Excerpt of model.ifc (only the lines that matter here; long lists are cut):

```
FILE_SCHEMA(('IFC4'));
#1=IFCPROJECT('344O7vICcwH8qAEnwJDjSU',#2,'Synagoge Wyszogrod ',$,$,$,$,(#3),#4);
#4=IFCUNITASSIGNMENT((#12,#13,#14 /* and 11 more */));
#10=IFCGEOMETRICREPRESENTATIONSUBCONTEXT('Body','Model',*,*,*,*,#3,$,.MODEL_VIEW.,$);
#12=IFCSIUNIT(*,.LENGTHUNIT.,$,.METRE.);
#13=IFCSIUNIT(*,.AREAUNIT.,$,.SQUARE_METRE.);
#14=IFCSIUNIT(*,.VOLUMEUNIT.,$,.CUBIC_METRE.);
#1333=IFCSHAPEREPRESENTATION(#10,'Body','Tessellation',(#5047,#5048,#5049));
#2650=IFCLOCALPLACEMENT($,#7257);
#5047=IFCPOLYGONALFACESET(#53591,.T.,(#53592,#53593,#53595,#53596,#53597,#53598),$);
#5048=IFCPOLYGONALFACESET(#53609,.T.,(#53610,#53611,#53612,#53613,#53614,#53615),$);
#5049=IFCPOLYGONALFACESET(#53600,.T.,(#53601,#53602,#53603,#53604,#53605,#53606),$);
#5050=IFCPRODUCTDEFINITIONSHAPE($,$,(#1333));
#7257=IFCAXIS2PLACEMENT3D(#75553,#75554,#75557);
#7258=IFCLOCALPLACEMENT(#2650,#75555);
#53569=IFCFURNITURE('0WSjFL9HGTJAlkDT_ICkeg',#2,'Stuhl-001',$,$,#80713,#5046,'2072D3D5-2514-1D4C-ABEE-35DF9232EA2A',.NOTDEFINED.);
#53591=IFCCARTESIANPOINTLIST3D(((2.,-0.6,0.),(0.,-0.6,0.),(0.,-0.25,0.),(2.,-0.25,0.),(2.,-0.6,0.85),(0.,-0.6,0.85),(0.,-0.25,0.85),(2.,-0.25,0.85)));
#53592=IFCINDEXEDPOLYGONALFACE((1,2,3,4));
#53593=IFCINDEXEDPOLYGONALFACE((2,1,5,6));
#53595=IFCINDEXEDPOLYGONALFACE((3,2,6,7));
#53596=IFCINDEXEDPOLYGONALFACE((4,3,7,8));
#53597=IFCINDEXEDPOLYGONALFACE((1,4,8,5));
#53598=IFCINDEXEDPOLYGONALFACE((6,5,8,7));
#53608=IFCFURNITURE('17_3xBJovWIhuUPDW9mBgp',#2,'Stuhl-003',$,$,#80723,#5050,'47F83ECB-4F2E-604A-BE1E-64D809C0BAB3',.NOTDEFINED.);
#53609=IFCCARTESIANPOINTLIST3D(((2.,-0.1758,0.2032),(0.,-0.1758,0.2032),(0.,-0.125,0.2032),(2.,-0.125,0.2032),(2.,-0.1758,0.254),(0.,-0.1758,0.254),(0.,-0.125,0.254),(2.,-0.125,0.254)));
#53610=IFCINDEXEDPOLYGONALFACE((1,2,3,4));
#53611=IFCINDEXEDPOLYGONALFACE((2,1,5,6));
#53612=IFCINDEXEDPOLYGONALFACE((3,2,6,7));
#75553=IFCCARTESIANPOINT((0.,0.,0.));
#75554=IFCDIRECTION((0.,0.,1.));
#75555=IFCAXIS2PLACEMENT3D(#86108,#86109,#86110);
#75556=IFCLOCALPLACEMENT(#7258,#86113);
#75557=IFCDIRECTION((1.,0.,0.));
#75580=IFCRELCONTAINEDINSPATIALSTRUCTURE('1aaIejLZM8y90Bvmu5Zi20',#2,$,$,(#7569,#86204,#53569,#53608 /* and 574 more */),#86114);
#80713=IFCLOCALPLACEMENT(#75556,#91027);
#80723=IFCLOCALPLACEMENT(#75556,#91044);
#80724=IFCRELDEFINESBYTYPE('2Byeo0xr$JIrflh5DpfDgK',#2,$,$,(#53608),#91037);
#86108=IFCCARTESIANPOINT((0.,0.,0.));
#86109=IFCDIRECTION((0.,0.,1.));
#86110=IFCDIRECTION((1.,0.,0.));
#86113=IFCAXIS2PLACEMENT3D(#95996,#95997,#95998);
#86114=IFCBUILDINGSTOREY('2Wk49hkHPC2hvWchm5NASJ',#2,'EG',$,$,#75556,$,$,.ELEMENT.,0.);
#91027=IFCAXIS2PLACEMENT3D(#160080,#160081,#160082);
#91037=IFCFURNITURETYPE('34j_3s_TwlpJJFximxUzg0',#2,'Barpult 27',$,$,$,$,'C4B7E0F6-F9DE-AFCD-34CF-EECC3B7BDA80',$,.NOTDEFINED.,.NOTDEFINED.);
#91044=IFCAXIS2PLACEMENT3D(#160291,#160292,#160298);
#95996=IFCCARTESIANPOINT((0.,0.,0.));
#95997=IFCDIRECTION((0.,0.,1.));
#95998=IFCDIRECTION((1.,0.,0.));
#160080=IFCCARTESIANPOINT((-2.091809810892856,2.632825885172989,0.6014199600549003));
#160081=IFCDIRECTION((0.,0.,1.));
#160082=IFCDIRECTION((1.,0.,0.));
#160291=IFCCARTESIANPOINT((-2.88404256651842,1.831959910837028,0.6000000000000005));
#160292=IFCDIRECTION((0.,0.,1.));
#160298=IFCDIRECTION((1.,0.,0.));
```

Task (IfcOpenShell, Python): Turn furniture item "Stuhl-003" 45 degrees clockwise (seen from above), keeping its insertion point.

```python
import ifcopenshell
import ifcopenshell.api.geometry
import ifcopenshell.util.placement

model = ifcopenshell.open("model.ifc")

item = model.by_guid("17_3xBJovWIhuUPDW9mBgp")
matrix = ifcopenshell.util.placement.get_local_placement(item.ObjectPlacement)
matrix = matrix @ ifcopenshell.util.placement.rotation(-45, "Z")
ifcopenshell.api.geometry.edit_object_placement(model, product=item, matrix=matrix, is_si=False)

print(ifcopenshell.util.placement.get_local_placement(item.ObjectPlacement).round(3) + 0.0)

model.write("model-out.ifc")
```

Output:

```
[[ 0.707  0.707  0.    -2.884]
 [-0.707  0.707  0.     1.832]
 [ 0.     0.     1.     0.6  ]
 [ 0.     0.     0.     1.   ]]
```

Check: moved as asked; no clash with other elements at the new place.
